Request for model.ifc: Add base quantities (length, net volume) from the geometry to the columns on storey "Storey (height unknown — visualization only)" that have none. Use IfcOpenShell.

First a look at what the model holds.

```python
import ifcopenshell
import ifcopenshell.util.element
import ifcopenshell.util.unit

model = ifcopenshell.open("model.ifc")
print(model.schema)
for unit_type in ("LENGTHUNIT", "AREAUNIT", "VOLUMEUNIT"):
    print(unit_type, ifcopenshell.util.unit.calculate_unit_scale(model, unit_type))
storey = next(s for s in model.by_type("IfcBuildingStorey") if s.Name == "Storey (height unknown — visualization only)")
columns = [e for e in ifcopenshell.util.element.get_decomposition(storey) if e.is_a("IfcColumn")]
for e in sorted(columns, key=lambda e: e.id()):
    print(e.id(), e.is_a(), e.Name, list(ifcopenshell.util.element.get_psets(e, qtos_only=True)), sep=" | ")
```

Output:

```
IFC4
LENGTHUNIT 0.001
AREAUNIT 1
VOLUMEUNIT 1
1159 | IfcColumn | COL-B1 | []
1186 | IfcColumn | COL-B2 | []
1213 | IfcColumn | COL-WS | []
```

```python
import ifcopenshell
import ifcopenshell.api.pset
import ifcopenshell.geom
import ifcopenshell.util.element
import ifcopenshell.util.shape
import ifcopenshell.util.unit

model = ifcopenshell.open("model.ifc")
unit_scale = ifcopenshell.util.unit.calculate_unit_scale(model)
volume_scale = ifcopenshell.util.unit.calculate_unit_scale(model, "VOLUMEUNIT")
settings = ifcopenshell.geom.settings()

storey = next(s for s in model.by_type("IfcBuildingStorey") if s.Name == "Storey (height unknown — visualization only)")
columns = [e for e in ifcopenshell.util.element.get_decomposition(storey) if e.is_a("IfcColumn")]

for e in sorted(columns, key=lambda e: e.id()):
    if ifcopenshell.util.element.get_psets(e, qtos_only=True, should_inherit=False):
        continue
    # Geometry comes back in metres, in the element's own axes.
    shape = ifcopenshell.geom.create_shape(settings, e)
    values = {
        "Length": ifcopenshell.util.shape.get_z(shape.geometry) / unit_scale,
        "NetVolume": ifcopenshell.util.shape.get_volume(shape.geometry) / volume_scale,
    }
    qto = ifcopenshell.api.pset.add_qto(model, product=e, name="Qto_ColumnBaseQuantities")
    ifcopenshell.api.pset.edit_qto(model, qto=qto, properties=values)
    print(e.id(), {k: round(v, 3) for k, v in values.items()})

model.write("model_updated.ifc")
```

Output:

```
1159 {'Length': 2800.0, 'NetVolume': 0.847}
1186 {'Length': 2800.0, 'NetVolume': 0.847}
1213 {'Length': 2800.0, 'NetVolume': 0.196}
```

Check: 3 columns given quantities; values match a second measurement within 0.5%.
